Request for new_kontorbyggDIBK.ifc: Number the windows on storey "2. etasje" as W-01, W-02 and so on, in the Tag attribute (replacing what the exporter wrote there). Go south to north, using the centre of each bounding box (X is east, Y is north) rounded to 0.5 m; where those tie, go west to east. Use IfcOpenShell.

First a look at what the model holds.

```python
import ifcopenshell
import ifcopenshell.util.element
import ifcopenshell.util.placement

model = ifcopenshell.open("new_kontorbyggDIBK.ifc")
print(model.schema)
storey = next(s for s in model.by_type("IfcBuildingStorey") if s.Name == "2. etasje")
windows = [e for e in ifcopenshell.util.element.get_decomposition(storey) if e.is_a("IfcWindow")]
for e in sorted(windows, key=lambda e: e.id()):
    origin = ifcopenshell.util.placement.get_local_placement(e.ObjectPlacement)[:3, 3]
    print(e.id(), e.Tag, e.Name, origin.round(2) + 0.0, sep=" | ")
```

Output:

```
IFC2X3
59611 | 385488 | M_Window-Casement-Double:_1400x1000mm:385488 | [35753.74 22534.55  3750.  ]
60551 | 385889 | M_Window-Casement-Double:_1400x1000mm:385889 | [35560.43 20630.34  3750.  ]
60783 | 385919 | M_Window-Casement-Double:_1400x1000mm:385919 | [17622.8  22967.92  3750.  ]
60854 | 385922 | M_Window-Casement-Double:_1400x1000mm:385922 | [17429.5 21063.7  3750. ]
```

```python
import ifcopenshell
import ifcopenshell.geom
import ifcopenshell.util.element
import ifcopenshell.util.shape

model = ifcopenshell.open("new_kontorbyggDIBK.ifc")
settings = ifcopenshell.geom.settings()
settings.set("use-world-coords", True)


def centre(element):
    shape = ifcopenshell.geom.create_shape(settings, element)
    return ifcopenshell.util.shape.get_bbox_centroid(shape.geometry)


storey = next(s for s in model.by_type("IfcBuildingStorey") if s.Name == "2. etasje")
windows = [e for e in ifcopenshell.util.element.get_decomposition(storey) if e.is_a("IfcWindow")]

# Insertion points can sit at a corner or the storey origin, so sort by the geometry (in metres).
centres = {e: centre(e) for e in windows}
windows.sort(key=lambda e: (round(centres[e][1] / 0.5), centres[e][0]))

for i, e in enumerate(windows, start=1):
    number = f"W-{i:02d}"
    e.Tag = number
    print(e.id(), number)

model.write("new_kontorbyggDIBK-out.ifc")
```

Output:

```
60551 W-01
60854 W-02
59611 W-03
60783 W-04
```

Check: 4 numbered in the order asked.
